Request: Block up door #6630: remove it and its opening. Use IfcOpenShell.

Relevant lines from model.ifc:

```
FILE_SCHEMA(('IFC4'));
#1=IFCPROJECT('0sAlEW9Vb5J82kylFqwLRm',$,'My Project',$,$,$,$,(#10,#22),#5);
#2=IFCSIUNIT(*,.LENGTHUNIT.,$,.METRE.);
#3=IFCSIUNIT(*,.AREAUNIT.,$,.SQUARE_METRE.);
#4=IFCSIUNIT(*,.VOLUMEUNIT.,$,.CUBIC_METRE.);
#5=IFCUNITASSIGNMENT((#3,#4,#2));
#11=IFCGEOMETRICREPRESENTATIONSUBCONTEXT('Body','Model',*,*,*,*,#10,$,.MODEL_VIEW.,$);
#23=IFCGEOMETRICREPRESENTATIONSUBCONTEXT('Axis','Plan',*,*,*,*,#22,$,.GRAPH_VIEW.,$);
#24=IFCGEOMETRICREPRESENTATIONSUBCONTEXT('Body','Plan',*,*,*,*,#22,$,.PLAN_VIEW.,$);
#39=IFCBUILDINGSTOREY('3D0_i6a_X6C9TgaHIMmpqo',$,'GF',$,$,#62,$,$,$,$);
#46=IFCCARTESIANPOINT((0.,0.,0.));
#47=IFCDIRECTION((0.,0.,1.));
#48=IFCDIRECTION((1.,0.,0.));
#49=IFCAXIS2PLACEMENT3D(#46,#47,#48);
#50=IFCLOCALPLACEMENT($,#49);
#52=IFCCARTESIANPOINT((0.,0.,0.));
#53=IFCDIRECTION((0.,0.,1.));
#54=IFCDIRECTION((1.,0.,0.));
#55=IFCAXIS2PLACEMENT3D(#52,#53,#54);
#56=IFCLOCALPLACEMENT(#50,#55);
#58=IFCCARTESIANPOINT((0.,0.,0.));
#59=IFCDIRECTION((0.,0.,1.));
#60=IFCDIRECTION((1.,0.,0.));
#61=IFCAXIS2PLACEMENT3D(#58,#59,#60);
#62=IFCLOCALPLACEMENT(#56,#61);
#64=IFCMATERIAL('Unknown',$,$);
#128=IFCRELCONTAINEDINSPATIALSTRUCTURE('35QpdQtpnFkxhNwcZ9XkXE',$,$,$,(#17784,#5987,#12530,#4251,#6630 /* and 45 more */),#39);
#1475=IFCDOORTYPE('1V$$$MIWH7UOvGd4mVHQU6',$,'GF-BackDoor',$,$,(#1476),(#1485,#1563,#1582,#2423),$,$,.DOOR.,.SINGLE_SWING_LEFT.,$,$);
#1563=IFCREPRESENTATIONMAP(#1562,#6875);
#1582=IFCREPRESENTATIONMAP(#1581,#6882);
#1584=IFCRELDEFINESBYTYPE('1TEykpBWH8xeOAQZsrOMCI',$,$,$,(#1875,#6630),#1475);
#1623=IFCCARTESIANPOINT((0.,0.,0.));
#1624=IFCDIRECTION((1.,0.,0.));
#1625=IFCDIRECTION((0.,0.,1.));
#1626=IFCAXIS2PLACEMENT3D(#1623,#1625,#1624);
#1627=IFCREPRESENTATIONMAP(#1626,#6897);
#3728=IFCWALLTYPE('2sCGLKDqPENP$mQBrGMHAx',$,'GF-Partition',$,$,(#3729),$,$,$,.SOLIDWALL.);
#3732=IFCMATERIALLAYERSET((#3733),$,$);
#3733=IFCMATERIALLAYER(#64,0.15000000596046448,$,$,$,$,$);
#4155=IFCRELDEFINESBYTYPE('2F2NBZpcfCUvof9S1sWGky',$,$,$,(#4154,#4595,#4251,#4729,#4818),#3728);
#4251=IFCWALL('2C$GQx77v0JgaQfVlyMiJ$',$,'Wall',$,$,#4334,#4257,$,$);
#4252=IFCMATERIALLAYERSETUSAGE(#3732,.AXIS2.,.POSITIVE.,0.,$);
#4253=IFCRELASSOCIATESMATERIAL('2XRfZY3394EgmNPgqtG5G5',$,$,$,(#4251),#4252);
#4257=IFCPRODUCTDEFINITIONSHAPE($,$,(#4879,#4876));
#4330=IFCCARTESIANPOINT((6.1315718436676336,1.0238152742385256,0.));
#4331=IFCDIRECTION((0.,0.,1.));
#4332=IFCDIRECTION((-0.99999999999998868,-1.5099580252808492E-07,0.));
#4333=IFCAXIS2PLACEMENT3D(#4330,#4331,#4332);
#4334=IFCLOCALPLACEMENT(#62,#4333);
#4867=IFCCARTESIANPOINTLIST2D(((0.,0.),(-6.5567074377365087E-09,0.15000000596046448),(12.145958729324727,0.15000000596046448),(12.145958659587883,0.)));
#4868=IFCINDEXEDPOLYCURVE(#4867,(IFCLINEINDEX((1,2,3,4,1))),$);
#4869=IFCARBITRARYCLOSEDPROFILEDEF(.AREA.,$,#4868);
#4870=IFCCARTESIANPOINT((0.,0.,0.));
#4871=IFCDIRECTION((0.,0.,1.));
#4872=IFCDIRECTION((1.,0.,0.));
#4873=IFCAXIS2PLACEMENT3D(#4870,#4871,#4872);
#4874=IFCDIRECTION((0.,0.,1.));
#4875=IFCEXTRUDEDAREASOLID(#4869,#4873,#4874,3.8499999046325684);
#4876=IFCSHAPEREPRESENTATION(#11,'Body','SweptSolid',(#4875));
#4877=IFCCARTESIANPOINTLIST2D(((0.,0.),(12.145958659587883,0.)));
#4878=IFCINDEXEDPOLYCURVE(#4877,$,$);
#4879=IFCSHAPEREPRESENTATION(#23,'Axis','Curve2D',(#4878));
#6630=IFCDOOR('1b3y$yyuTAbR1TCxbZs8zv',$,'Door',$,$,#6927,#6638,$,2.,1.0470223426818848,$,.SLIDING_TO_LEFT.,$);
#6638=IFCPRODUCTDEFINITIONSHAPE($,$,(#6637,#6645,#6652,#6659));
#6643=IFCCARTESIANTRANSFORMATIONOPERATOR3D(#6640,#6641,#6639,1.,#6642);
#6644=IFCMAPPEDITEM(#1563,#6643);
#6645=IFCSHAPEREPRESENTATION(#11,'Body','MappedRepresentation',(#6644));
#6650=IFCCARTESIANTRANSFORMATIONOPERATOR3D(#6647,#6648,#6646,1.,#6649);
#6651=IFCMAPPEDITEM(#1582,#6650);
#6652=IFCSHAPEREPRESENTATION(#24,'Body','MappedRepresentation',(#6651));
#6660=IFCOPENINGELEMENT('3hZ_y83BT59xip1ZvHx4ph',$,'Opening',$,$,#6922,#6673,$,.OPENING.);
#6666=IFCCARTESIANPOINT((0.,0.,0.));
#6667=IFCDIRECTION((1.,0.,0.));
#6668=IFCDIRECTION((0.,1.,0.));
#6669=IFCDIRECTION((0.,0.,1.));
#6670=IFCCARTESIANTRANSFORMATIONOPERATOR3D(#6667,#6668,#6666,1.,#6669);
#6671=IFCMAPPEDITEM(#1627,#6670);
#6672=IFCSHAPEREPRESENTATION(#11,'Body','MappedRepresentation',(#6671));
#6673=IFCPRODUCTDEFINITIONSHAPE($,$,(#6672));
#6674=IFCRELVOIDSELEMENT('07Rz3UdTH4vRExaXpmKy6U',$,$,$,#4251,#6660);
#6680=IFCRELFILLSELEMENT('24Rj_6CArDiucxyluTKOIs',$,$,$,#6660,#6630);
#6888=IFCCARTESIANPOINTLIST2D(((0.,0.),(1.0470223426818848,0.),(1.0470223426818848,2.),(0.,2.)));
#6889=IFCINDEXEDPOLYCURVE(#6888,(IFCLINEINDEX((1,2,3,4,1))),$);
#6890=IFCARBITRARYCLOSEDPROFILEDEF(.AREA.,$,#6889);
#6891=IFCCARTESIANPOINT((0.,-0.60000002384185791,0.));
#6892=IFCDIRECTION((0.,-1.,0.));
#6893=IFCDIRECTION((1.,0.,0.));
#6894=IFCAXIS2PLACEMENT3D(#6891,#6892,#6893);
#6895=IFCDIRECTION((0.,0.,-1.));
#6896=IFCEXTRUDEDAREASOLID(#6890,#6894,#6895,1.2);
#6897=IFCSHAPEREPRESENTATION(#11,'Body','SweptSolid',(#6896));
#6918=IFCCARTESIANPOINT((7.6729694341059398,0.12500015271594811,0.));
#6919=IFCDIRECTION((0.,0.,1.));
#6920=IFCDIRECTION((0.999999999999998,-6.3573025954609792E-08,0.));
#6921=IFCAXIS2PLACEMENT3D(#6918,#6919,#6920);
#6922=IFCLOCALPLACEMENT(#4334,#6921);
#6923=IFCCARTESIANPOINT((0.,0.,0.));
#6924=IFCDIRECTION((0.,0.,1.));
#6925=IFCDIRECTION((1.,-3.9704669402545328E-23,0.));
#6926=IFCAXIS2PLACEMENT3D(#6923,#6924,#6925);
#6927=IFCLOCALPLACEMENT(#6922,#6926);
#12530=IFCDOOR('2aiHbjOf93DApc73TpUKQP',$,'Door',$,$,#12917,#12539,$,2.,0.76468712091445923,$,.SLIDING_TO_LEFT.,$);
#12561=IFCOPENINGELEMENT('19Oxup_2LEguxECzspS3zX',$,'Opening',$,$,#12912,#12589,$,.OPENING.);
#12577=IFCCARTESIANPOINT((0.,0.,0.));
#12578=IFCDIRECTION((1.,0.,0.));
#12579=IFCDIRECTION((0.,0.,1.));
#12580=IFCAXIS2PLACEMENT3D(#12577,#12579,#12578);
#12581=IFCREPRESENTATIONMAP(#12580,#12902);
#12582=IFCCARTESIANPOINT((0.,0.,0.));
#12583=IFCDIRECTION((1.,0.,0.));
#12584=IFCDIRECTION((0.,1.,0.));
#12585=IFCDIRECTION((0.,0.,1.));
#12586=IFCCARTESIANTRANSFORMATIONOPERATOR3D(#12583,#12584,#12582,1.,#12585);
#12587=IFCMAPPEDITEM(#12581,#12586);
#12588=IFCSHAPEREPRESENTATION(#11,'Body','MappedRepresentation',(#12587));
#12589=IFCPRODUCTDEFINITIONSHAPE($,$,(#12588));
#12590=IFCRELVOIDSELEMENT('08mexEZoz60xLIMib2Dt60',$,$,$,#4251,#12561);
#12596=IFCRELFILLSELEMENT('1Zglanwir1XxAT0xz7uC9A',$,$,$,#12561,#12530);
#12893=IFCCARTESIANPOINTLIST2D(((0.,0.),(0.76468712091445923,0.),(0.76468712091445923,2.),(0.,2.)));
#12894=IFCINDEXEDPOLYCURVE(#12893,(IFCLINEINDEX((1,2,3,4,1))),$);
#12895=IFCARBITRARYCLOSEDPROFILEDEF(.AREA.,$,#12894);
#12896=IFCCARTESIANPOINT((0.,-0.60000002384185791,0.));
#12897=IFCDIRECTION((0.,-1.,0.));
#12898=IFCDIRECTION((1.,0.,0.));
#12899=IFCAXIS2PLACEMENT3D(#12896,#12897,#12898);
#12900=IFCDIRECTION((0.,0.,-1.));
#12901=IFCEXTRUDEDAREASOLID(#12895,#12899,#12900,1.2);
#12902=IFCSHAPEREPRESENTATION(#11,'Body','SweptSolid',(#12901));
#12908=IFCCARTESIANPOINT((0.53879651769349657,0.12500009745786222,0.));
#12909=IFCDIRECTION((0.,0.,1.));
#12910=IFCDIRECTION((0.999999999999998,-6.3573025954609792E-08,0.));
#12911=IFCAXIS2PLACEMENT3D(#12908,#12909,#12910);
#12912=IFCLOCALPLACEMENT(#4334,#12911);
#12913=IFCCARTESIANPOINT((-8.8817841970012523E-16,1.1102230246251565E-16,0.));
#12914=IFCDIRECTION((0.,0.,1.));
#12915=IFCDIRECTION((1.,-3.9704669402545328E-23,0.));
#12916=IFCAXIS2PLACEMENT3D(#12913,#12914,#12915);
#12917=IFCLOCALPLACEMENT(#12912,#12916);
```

```python
import ifcopenshell
import ifcopenshell.api.feature
import ifcopenshell.api.root
import ifcopenshell.geom
import ifcopenshell.util.shape

model = ifcopenshell.open("model.ifc")
settings = ifcopenshell.geom.settings()


def volume(element):
    """Net volume in cubic metres, openings subtracted."""
    shape = ifcopenshell.geom.create_shape(settings, element)
    return ifcopenshell.util.shape.get_volume(shape.geometry)


door = model.by_guid("1b3y$yyuTAbR1TCxbZs8zv")
opening = door.FillsVoids[0].RelatingOpeningElement
wall = opening.VoidsElements[0].RelatingBuildingElement
before = volume(wall)

ifcopenshell.api.root.remove_product(model, product=door)
ifcopenshell.api.feature.remove_feature(model, feature=opening)

after = volume(wall)

print(f"wall volume {before:.3f} -> {after:.3f} m3")

model.write("model_edited.ifc")
```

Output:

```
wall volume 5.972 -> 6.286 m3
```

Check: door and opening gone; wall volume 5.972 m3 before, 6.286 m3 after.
